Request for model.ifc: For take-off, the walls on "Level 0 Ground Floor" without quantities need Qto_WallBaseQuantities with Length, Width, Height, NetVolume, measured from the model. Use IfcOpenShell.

First a look at what the model holds.

```python
import ifcopenshell
import ifcopenshell.util.element
import ifcopenshell.util.unit

model = ifcopenshell.open("model.ifc")
print(model.schema)
for unit_type in ("LENGTHUNIT", "AREAUNIT", "VOLUMEUNIT"):
    print(unit_type, ifcopenshell.util.unit.calculate_unit_scale(model, unit_type))
storey = next(s for s in model.by_type("IfcBuildingStorey") if s.Name == "Level 0 Ground Floor")
walls = [e for e in ifcopenshell.util.element.get_decomposition(storey) if e.is_a("IfcWall")]
for e in sorted(walls, key=lambda e: e.id()):
    print(e.id(), e.is_a(), e.Name, list(ifcopenshell.util.element.get_psets(e, qtos_only=True)), sep=" | ")
```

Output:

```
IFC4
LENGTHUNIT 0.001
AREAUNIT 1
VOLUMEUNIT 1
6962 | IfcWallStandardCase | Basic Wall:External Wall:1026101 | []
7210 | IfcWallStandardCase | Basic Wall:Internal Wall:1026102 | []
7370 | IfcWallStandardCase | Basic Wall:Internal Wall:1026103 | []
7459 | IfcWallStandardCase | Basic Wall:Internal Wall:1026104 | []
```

```python
import ifcopenshell
import ifcopenshell.api.pset
import ifcopenshell.geom
import ifcopenshell.util.element
import ifcopenshell.util.shape
import ifcopenshell.util.unit

model = ifcopenshell.open("model.ifc")
unit_scale = ifcopenshell.util.unit.calculate_unit_scale(model)
volume_scale = ifcopenshell.util.unit.calculate_unit_scale(model, "VOLUMEUNIT")
settings = ifcopenshell.geom.settings()

storey = next(s for s in model.by_type("IfcBuildingStorey") if s.Name == "Level 0 Ground Floor")
walls = [e for e in ifcopenshell.util.element.get_decomposition(storey) if e.is_a("IfcWall")]

for e in sorted(walls, key=lambda e: e.id()):
    if ifcopenshell.util.element.get_psets(e, qtos_only=True, should_inherit=False):
        continue
    # Geometry comes back in metres, in the element's own axes.
    shape = ifcopenshell.geom.create_shape(settings, e)
    values = {
        "Length": ifcopenshell.util.shape.get_x(shape.geometry) / unit_scale,
        "Width": ifcopenshell.util.shape.get_y(shape.geometry) / unit_scale,
        "Height": ifcopenshell.util.shape.get_z(shape.geometry) / unit_scale,
        "NetVolume": ifcopenshell.util.shape.get_volume(shape.geometry) / volume_scale,
    }
    qto = ifcopenshell.api.pset.add_qto(model, product=e, name="Qto_WallBaseQuantities")
    ifcopenshell.api.pset.edit_qto(model, qto=qto, properties=values)
    print(e.id(), {k: round(v, 3) for k, v in values.items()})

model.write("model_edited.ifc")
```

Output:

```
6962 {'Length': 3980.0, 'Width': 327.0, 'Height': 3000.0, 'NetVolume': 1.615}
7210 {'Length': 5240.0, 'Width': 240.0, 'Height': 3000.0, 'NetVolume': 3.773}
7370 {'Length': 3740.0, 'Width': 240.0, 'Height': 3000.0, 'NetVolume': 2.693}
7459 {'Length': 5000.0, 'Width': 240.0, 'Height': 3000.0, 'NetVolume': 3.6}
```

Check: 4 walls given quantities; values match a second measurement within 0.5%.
